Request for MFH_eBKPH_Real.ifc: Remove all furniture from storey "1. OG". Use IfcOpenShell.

First a look at what the model holds.

```python
import ifcopenshell
import ifcopenshell.util.element

model = ifcopenshell.open("MFH_eBKPH_Real.ifc")
print(model.schema)
storey = next(s for s in model.by_type("IfcBuildingStorey") if s.Name == "1. OG")
furniture = [e for e in ifcopenshell.util.element.get_decomposition(storey) if e.is_a("IfcFurnishingElement")]
seen = {}
for e in furniture:
    element_type = ifcopenshell.util.element.get_type(e)
    name = element_type.Name if element_type not in (None, e) else None
    seen[name] = seen.get(name, 0) + 1
for name, count in sorted(seen.items(), key=str):
    print(count, "x", name)
```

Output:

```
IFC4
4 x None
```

```python
import ifcopenshell
import ifcopenshell.api.root
import ifcopenshell.util.element

model = ifcopenshell.open("MFH_eBKPH_Real.ifc")

storey = next(s for s in model.by_type("IfcBuildingStorey") if s.Name == "1. OG")
furniture = [e for e in ifcopenshell.util.element.get_decomposition(storey) if e.is_a("IfcFurnishingElement")]

for e in furniture:
    ifcopenshell.api.root.remove_product(model, product=e)
print(len(furniture), "removed")

model.write("MFH_eBKPH_Real_v2.ifc")
```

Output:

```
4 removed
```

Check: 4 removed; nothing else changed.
